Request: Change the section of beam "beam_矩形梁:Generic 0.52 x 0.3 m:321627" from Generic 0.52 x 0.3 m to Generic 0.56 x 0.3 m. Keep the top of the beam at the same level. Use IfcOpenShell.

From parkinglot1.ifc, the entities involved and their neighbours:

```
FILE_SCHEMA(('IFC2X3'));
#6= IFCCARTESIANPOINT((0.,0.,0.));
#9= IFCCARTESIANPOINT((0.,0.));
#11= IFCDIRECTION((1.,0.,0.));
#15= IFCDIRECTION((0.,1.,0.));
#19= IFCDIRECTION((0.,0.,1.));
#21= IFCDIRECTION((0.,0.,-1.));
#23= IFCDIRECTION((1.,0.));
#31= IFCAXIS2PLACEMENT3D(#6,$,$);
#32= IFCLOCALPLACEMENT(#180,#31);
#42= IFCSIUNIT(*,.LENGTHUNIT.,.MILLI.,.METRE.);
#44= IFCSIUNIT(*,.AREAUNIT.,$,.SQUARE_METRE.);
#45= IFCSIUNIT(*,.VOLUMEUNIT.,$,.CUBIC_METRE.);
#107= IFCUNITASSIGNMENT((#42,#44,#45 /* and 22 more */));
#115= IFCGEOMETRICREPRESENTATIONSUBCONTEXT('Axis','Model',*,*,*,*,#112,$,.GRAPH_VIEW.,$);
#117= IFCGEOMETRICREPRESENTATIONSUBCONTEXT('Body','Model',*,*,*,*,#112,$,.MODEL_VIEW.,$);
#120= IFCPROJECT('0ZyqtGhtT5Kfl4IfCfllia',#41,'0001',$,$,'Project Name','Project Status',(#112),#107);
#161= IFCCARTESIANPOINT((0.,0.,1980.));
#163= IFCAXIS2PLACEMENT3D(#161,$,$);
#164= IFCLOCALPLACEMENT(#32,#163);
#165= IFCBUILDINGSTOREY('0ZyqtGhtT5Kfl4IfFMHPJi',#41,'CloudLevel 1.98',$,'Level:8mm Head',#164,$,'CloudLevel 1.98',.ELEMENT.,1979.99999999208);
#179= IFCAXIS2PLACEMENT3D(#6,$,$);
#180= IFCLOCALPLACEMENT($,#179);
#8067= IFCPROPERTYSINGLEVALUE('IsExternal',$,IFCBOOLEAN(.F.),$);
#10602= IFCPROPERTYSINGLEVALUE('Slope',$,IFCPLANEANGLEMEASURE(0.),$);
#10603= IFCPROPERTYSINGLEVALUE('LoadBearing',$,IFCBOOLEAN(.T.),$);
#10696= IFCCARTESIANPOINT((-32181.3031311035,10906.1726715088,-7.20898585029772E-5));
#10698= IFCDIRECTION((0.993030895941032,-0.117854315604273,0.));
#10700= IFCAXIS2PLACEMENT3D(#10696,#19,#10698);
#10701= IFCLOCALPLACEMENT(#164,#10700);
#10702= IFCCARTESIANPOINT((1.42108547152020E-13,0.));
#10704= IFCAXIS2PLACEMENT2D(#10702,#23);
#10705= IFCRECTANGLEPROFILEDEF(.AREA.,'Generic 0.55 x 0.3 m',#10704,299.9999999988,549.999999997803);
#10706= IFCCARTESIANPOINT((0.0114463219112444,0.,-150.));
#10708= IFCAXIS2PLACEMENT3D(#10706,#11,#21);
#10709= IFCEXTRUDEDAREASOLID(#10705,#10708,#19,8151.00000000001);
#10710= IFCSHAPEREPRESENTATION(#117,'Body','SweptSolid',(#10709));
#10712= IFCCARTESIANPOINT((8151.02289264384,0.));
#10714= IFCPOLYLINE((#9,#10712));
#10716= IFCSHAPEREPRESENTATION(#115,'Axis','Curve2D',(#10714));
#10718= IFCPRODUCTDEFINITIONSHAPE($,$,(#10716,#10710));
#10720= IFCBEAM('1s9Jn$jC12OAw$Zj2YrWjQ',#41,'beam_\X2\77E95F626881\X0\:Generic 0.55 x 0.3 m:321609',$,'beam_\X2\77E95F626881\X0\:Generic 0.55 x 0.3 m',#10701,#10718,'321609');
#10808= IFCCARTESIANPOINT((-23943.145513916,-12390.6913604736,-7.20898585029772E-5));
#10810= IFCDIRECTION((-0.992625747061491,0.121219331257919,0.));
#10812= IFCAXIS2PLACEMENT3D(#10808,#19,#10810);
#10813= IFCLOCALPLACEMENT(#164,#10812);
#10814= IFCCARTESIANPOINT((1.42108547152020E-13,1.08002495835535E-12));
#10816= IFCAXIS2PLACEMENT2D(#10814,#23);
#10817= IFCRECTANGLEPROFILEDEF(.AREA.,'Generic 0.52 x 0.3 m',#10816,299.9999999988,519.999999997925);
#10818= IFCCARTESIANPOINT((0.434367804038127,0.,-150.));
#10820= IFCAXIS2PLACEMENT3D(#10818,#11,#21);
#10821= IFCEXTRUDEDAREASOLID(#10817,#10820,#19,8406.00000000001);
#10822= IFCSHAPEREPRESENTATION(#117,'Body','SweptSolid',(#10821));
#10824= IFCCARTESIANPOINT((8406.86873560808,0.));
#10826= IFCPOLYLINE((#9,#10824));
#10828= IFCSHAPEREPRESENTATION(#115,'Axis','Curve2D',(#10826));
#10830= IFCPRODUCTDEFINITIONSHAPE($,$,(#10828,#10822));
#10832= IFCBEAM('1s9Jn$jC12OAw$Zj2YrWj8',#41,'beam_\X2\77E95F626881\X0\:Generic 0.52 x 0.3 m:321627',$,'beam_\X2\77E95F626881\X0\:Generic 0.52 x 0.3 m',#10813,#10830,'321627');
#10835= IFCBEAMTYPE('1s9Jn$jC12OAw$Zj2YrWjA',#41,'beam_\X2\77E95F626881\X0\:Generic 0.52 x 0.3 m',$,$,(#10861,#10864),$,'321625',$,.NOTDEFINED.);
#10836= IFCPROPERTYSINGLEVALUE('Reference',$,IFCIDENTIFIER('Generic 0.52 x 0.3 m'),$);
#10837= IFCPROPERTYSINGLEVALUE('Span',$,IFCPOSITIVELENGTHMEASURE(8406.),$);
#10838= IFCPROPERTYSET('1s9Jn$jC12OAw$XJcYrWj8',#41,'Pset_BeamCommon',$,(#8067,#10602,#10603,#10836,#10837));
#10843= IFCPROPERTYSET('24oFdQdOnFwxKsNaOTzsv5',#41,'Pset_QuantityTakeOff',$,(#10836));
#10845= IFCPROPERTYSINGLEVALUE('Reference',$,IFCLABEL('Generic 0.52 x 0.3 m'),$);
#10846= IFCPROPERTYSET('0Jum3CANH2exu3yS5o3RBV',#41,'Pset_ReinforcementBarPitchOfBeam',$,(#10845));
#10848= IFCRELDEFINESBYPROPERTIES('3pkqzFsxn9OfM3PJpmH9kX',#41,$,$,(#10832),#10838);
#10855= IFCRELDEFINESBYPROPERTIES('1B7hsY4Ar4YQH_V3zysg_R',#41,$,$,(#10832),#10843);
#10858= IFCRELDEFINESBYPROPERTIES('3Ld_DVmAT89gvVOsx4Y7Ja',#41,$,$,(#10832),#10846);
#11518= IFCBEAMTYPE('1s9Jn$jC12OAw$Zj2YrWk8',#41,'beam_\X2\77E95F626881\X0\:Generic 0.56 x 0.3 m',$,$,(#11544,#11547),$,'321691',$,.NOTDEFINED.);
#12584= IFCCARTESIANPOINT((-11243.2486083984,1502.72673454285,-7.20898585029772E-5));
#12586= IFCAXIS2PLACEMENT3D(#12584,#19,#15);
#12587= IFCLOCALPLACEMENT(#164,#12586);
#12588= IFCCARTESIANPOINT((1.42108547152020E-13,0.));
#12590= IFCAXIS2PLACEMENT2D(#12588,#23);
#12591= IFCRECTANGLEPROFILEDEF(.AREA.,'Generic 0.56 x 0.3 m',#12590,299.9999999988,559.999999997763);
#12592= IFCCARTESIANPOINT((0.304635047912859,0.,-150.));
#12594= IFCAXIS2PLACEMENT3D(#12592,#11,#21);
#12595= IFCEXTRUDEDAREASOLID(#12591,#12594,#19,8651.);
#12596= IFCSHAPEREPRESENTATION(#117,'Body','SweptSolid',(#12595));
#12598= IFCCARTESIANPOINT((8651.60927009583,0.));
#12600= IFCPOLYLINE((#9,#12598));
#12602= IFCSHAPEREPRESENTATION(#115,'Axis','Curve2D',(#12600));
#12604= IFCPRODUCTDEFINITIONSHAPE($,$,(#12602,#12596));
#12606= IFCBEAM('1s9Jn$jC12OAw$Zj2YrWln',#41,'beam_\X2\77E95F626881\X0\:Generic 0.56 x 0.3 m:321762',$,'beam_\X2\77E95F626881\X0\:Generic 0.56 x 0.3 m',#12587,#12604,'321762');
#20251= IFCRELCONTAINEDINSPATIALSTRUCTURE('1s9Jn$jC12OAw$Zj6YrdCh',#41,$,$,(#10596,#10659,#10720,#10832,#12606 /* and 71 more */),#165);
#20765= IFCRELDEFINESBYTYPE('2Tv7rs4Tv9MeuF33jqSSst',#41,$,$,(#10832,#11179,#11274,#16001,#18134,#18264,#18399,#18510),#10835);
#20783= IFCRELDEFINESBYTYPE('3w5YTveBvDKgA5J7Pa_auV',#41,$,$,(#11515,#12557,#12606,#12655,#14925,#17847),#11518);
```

```python
import ifcopenshell
import ifcopenshell.api.pset
import ifcopenshell.api.type
import ifcopenshell.util.element
import ifcopenshell.util.representation

model = ifcopenshell.open("parkinglot1.ifc")

member = model.by_guid("1s9Jn$jC12OAw$Zj2YrWj8")
source = next(p for p in model.by_type("IfcRectangleProfileDef") if p.ProfileName == "Generic 0.56 x 0.3 m")

body = ifcopenshell.util.representation.get_representation(member, "Model", "Body")
solid = body.Items[0]
old_profile = solid.SweptArea

# Copy the section's sizes but keep this member's own profile position.
profile = ifcopenshell.util.element.copy(model, source)
# Profiles are centred, so shift by half the change in depth to hold the top.
shift = (old_profile.XDim - profile.XDim) / 2
x, y = old_profile.Position.Location.Coordinates
up = (-1.0, 0.0)  # upwards, in the solid's own plane
location = model.createIfcCartesianPoint((x + up[0] * shift, y + up[1] * shift))
profile.Position = model.createIfcAxis2Placement2D(location, old_profile.Position.RefDirection)
solid.SweptArea = profile
if not model.get_total_inverses(old_profile):
    ifcopenshell.util.element.remove_deep2(model, old_profile)

new_type = model.by_id(11518)
ifcopenshell.api.type.assign_type(
    model, related_objects=[member], relating_type=new_type, should_map_representations=False
)
member.Name = member.Name.replace("Generic 0.52 x 0.3 m", "Generic 0.56 x 0.3 m")
member.ObjectType = "beam_矩形梁:Generic 0.56 x 0.3 m"
pset = model.by_id(ifcopenshell.util.element.get_pset(member, "Pset_BeamCommon", should_inherit=False)["id"])
ifcopenshell.api.pset.edit_pset(model, pset=pset, properties={"Reference": "Generic 0.56 x 0.3 m"})
pset = model.by_id(ifcopenshell.util.element.get_pset(member, "Pset_QuantityTakeOff", should_inherit=False)["id"])
ifcopenshell.api.pset.edit_pset(model, pset=pset, properties={"Reference": "Generic 0.56 x 0.3 m"})
pset = model.by_id(ifcopenshell.util.element.get_pset(member, "Pset_ReinforcementBarPitchOfBeam", should_inherit=False)["id"])
ifcopenshell.api.pset.edit_pset(model, pset=pset, properties={"Reference": "Generic 0.56 x 0.3 m"})

print(solid.SweptArea)

model.write("parkinglot1_updated.ifc")
```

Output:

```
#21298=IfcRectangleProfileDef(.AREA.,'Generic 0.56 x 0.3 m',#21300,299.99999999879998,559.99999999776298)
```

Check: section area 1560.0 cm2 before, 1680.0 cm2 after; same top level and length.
